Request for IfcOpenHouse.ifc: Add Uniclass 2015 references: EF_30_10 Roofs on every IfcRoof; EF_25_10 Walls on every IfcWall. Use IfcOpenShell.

First a look at what the model holds.

```python
import ifcopenshell

model = ifcopenshell.open("IfcOpenHouse.ifc")
print(model.schema)
print("classifications:", [c.Name for c in model.by_type("IfcClassification")])
for ifc_class in ("IfcDoor", "IfcRoof", "IfcStair", "IfcWall", "IfcWindow"):
    print(ifc_class, len(model.by_type(ifc_class)))
```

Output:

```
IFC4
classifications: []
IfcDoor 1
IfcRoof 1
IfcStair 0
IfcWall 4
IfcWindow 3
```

```python
import ifcopenshell
import ifcopenshell.api.classification

model = ifcopenshell.open("IfcOpenHouse.ifc")

system = ifcopenshell.api.classification.add_classification(model, classification="Uniclass 2015")

codes = {
    "IfcRoof": ("EF_30_10", "Roofs"),
    "IfcWall": ("EF_25_10", "Walls"),
}
for ifc_class, (code, name) in codes.items():
    products = model.by_type(ifc_class)
    ifcopenshell.api.classification.add_reference(
        model, products=products, classification=system, identification=code, name=name
    )
    print(code, len(products))

model.write("IfcOpenHouse_updated.ifc")
```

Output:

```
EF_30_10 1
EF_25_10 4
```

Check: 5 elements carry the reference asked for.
